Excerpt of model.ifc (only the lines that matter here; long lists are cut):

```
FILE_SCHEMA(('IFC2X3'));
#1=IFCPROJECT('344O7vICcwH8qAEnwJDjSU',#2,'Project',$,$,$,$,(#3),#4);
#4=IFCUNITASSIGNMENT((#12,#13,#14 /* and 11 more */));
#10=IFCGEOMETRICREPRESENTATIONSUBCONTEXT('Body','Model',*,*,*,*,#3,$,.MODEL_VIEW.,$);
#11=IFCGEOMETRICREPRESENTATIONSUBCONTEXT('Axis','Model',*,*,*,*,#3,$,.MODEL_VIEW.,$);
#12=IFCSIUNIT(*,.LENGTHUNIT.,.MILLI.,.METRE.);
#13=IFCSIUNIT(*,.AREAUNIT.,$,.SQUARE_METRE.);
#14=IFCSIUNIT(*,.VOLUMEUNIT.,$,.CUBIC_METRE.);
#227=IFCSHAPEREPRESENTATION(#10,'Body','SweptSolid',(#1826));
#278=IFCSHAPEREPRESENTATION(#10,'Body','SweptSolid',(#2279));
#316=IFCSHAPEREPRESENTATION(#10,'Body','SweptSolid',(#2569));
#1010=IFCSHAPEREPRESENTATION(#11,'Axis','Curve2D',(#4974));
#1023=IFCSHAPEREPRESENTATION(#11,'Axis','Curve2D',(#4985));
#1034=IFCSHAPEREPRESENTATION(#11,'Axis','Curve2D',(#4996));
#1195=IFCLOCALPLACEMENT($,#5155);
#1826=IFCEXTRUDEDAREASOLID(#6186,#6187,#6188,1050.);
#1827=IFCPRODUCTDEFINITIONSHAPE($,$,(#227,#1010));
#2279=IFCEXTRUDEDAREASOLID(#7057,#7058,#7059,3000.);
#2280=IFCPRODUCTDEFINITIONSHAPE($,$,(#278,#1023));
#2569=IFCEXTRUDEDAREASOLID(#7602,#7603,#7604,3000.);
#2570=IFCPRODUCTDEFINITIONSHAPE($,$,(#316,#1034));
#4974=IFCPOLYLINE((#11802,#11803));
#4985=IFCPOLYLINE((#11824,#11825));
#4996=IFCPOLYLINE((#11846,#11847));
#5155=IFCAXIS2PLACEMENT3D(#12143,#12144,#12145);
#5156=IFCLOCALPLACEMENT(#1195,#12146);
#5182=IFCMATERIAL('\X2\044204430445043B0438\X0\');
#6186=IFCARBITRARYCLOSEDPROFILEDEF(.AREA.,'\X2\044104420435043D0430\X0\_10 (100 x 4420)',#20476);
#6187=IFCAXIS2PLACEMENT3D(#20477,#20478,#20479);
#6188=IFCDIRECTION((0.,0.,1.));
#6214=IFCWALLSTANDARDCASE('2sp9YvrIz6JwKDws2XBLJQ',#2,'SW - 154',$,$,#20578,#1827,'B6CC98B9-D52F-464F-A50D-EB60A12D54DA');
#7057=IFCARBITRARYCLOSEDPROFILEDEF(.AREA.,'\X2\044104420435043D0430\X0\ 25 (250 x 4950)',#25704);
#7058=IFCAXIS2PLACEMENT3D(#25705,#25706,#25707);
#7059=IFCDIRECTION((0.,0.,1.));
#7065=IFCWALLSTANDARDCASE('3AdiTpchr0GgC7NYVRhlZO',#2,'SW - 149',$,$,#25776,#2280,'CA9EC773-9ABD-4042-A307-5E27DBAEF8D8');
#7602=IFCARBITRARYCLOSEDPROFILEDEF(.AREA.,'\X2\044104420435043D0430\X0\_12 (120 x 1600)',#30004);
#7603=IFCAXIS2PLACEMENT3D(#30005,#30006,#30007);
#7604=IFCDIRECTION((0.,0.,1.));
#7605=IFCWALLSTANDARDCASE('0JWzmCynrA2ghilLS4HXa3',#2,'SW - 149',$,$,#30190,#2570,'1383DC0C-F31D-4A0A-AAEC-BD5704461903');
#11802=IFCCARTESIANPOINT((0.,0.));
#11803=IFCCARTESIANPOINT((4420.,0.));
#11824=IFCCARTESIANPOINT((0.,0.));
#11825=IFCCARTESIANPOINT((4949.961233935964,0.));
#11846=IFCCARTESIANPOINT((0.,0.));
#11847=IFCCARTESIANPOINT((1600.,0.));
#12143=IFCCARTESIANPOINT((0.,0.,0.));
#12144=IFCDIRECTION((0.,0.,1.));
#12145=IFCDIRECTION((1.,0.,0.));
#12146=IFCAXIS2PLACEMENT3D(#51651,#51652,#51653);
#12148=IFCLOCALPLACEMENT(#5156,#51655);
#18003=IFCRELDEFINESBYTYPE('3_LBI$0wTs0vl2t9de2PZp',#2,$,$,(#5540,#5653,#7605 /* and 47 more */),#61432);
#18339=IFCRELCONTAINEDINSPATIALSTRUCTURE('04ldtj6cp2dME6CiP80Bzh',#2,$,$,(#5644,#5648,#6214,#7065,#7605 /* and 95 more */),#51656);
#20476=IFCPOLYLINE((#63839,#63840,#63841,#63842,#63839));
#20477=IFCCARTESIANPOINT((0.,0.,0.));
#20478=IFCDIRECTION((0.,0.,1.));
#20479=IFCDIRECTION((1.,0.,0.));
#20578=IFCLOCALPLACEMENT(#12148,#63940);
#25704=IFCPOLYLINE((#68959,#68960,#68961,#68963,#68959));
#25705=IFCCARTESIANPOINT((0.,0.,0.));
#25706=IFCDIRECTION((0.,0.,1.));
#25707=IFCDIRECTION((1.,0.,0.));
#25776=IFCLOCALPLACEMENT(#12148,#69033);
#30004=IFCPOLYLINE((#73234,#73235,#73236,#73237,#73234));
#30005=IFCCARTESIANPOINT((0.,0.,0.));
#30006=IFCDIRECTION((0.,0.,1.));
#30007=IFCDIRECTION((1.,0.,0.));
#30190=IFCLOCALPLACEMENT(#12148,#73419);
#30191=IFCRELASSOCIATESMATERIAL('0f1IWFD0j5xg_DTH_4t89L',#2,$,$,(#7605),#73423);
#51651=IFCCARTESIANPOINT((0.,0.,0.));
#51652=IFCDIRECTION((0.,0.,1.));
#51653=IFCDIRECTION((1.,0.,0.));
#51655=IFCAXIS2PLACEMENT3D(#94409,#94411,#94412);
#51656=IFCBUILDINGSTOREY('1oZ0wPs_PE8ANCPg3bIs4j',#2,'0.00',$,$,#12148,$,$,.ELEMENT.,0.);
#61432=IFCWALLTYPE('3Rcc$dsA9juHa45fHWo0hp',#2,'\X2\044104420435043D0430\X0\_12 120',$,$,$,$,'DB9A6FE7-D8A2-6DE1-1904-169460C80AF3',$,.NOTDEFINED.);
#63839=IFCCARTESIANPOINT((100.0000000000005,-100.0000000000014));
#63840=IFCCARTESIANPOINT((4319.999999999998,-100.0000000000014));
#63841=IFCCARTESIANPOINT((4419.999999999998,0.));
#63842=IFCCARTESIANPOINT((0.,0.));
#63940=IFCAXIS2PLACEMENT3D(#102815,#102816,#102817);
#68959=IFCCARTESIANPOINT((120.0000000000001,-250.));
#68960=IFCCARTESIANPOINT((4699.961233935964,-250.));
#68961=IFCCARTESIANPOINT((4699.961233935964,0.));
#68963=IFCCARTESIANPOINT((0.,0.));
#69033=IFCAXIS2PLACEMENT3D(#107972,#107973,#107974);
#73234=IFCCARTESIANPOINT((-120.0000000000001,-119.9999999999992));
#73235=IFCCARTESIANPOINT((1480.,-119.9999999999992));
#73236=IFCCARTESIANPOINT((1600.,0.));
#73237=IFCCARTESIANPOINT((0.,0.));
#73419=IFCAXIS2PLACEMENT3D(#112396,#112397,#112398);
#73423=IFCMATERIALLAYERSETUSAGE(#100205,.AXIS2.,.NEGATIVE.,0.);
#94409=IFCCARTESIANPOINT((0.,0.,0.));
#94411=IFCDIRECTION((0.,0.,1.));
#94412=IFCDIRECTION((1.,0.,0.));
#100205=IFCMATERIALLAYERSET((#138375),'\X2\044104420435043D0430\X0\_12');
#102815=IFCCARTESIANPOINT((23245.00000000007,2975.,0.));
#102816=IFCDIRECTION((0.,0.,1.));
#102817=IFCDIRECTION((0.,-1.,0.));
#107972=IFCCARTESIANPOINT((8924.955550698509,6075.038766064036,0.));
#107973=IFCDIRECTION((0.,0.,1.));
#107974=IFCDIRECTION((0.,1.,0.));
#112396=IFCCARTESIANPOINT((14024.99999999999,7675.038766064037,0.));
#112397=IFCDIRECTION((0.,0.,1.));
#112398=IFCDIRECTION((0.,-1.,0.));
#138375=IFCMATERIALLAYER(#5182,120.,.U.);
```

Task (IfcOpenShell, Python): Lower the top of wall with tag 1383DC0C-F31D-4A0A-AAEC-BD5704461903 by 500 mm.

```python
import ifcopenshell
import ifcopenshell.geom
import ifcopenshell.util.representation
import ifcopenshell.util.shape

model = ifcopenshell.open("model.ifc")
settings = ifcopenshell.geom.settings()


def volume(element):
    """Net volume in cubic metres, openings subtracted."""
    shape = ifcopenshell.geom.create_shape(settings, element)
    return ifcopenshell.util.shape.get_volume(shape.geometry)


wall = model.by_guid("0JWzmCynrA2ghilLS4HXa3")
before = volume(wall)

body = ifcopenshell.util.representation.get_representation(wall, "Model", "Body")
solid = body.Items[0]
old_height = solid.Depth
solid.Depth -= 500.0
after = volume(wall)

print(f"height {old_height:g} -> {solid.Depth:g}, volume {before:.3f} -> {after:.3f} m3")

model.write("model_rev.ifc")
```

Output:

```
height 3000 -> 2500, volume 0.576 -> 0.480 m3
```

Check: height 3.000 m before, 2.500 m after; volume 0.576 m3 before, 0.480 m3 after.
